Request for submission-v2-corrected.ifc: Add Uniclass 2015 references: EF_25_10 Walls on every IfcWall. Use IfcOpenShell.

First a look at what the model holds.

```python
import ifcopenshell

model = ifcopenshell.open("submission-v2-corrected.ifc")
print(model.schema)
print("classifications:", [c.Name for c in model.by_type("IfcClassification")])
for ifc_class in ("IfcDoor", "IfcRoof", "IfcStair", "IfcWall", "IfcWindow"):
    print(ifc_class, len(model.by_type(ifc_class)))
```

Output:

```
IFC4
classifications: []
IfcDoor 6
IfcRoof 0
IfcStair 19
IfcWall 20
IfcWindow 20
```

```python
import ifcopenshell
import ifcopenshell.api.classification

model = ifcopenshell.open("submission-v2-corrected.ifc")

system = ifcopenshell.api.classification.add_classification(model, classification="Uniclass 2015")

codes = {
    "IfcWall": ("EF_25_10", "Walls"),
}
for ifc_class, (code, name) in codes.items():
    products = model.by_type(ifc_class)
    ifcopenshell.api.classification.add_reference(
        model, products=products, classification=system, identification=code, name=name
    )
    print(code, len(products))

model.write("submission-v2-corrected_updated.ifc")
```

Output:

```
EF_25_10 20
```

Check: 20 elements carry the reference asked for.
